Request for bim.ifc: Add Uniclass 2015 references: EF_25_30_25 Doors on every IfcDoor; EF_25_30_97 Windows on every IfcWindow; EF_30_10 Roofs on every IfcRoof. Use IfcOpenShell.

First a look at what the model holds.

```python
import ifcopenshell

model = ifcopenshell.open("bim.ifc")
print(model.schema)
print("classifications:", [c.Name for c in model.by_type("IfcClassification")])
for ifc_class in ("IfcDoor", "IfcRoof", "IfcStair", "IfcWall", "IfcWindow"):
    print(ifc_class, len(model.by_type(ifc_class)))
```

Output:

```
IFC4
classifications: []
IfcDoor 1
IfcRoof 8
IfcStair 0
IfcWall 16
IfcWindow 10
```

```python
import ifcopenshell
import ifcopenshell.api.classification

model = ifcopenshell.open("bim.ifc")

system = ifcopenshell.api.classification.add_classification(model, classification="Uniclass 2015")

codes = {
    "IfcDoor": ("EF_25_30_25", "Doors"),
    "IfcWindow": ("EF_25_30_97", "Windows"),
    "IfcRoof": ("EF_30_10", "Roofs"),
}
for ifc_class, (code, name) in codes.items():
    products = model.by_type(ifc_class)
    ifcopenshell.api.classification.add_reference(
        model, products=products, classification=system, identification=code, name=name
    )
    print(code, len(products))

model.write("bim_rev.ifc")
```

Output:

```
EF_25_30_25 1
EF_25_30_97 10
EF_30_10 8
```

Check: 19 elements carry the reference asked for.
